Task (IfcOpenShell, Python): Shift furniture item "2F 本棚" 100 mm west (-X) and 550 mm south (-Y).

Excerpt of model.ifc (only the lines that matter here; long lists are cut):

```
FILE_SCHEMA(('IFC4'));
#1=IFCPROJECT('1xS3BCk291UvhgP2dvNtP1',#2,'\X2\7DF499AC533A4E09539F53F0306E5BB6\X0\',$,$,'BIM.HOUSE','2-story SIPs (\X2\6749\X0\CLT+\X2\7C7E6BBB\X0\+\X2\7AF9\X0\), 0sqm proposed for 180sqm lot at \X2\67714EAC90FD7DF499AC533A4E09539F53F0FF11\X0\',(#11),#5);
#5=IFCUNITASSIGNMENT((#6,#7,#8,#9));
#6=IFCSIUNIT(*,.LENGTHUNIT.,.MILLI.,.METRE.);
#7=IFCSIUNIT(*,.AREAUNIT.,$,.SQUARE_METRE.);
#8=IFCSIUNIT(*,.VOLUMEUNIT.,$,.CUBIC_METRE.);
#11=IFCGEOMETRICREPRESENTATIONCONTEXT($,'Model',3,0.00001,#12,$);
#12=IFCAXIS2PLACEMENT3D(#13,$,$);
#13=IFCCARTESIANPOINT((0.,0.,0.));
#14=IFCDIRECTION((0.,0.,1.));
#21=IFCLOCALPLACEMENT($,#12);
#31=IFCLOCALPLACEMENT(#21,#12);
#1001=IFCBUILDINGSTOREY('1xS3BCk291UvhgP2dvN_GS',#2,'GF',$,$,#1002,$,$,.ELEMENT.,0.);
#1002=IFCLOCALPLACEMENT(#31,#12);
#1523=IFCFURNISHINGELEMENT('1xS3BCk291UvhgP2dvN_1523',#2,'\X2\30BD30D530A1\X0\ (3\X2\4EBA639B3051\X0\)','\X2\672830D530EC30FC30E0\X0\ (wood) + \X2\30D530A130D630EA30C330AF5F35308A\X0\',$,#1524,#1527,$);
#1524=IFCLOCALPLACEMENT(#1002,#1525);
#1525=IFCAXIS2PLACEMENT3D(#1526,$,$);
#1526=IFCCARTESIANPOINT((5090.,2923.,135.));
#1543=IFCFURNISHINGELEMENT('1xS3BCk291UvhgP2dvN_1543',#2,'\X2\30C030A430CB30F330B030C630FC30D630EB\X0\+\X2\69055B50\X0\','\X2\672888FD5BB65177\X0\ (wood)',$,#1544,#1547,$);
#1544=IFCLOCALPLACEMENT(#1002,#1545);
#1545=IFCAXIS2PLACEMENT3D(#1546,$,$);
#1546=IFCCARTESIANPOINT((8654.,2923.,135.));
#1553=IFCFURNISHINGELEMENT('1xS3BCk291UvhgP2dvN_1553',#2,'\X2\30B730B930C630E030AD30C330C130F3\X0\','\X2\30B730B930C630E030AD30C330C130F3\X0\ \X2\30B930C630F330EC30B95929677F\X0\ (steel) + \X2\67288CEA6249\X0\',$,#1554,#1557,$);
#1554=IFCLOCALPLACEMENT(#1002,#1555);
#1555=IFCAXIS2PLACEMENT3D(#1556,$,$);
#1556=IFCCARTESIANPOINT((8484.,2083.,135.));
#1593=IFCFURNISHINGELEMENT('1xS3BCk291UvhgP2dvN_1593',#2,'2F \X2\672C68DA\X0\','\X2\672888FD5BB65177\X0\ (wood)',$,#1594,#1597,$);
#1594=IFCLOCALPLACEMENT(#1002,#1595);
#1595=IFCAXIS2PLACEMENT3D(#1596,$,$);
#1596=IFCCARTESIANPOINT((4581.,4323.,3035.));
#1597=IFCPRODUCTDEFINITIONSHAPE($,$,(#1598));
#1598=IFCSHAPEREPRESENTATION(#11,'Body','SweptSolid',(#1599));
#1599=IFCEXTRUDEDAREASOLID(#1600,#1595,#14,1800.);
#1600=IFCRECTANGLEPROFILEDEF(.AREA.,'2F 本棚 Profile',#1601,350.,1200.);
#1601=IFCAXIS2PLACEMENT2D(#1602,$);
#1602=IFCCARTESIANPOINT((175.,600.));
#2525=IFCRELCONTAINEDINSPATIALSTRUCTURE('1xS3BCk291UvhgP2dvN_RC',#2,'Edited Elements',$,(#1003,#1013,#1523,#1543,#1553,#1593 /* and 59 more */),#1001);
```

```python
import ifcopenshell
import ifcopenshell.api.geometry
import ifcopenshell.util.placement
import ifcopenshell.util.unit

model = ifcopenshell.open("model.ifc")
unit_scale = ifcopenshell.util.unit.calculate_unit_scale(model)

item = model.by_guid("1xS3BCk291UvhgP2dvN_1593")
matrix = ifcopenshell.util.placement.get_local_placement(item.ObjectPlacement)
matrix[0, 3] -= 0.1 / unit_scale
matrix[1, 3] -= 0.55 / unit_scale
ifcopenshell.api.geometry.edit_object_placement(model, product=item, matrix=matrix, is_si=False)

print(ifcopenshell.util.placement.get_local_placement(item.ObjectPlacement).round(3) + 0.0)

model.write("model_rev.ifc")
```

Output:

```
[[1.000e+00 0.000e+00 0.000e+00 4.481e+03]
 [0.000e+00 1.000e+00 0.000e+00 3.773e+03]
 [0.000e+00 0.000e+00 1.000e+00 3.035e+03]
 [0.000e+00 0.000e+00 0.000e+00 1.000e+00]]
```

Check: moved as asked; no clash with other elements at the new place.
